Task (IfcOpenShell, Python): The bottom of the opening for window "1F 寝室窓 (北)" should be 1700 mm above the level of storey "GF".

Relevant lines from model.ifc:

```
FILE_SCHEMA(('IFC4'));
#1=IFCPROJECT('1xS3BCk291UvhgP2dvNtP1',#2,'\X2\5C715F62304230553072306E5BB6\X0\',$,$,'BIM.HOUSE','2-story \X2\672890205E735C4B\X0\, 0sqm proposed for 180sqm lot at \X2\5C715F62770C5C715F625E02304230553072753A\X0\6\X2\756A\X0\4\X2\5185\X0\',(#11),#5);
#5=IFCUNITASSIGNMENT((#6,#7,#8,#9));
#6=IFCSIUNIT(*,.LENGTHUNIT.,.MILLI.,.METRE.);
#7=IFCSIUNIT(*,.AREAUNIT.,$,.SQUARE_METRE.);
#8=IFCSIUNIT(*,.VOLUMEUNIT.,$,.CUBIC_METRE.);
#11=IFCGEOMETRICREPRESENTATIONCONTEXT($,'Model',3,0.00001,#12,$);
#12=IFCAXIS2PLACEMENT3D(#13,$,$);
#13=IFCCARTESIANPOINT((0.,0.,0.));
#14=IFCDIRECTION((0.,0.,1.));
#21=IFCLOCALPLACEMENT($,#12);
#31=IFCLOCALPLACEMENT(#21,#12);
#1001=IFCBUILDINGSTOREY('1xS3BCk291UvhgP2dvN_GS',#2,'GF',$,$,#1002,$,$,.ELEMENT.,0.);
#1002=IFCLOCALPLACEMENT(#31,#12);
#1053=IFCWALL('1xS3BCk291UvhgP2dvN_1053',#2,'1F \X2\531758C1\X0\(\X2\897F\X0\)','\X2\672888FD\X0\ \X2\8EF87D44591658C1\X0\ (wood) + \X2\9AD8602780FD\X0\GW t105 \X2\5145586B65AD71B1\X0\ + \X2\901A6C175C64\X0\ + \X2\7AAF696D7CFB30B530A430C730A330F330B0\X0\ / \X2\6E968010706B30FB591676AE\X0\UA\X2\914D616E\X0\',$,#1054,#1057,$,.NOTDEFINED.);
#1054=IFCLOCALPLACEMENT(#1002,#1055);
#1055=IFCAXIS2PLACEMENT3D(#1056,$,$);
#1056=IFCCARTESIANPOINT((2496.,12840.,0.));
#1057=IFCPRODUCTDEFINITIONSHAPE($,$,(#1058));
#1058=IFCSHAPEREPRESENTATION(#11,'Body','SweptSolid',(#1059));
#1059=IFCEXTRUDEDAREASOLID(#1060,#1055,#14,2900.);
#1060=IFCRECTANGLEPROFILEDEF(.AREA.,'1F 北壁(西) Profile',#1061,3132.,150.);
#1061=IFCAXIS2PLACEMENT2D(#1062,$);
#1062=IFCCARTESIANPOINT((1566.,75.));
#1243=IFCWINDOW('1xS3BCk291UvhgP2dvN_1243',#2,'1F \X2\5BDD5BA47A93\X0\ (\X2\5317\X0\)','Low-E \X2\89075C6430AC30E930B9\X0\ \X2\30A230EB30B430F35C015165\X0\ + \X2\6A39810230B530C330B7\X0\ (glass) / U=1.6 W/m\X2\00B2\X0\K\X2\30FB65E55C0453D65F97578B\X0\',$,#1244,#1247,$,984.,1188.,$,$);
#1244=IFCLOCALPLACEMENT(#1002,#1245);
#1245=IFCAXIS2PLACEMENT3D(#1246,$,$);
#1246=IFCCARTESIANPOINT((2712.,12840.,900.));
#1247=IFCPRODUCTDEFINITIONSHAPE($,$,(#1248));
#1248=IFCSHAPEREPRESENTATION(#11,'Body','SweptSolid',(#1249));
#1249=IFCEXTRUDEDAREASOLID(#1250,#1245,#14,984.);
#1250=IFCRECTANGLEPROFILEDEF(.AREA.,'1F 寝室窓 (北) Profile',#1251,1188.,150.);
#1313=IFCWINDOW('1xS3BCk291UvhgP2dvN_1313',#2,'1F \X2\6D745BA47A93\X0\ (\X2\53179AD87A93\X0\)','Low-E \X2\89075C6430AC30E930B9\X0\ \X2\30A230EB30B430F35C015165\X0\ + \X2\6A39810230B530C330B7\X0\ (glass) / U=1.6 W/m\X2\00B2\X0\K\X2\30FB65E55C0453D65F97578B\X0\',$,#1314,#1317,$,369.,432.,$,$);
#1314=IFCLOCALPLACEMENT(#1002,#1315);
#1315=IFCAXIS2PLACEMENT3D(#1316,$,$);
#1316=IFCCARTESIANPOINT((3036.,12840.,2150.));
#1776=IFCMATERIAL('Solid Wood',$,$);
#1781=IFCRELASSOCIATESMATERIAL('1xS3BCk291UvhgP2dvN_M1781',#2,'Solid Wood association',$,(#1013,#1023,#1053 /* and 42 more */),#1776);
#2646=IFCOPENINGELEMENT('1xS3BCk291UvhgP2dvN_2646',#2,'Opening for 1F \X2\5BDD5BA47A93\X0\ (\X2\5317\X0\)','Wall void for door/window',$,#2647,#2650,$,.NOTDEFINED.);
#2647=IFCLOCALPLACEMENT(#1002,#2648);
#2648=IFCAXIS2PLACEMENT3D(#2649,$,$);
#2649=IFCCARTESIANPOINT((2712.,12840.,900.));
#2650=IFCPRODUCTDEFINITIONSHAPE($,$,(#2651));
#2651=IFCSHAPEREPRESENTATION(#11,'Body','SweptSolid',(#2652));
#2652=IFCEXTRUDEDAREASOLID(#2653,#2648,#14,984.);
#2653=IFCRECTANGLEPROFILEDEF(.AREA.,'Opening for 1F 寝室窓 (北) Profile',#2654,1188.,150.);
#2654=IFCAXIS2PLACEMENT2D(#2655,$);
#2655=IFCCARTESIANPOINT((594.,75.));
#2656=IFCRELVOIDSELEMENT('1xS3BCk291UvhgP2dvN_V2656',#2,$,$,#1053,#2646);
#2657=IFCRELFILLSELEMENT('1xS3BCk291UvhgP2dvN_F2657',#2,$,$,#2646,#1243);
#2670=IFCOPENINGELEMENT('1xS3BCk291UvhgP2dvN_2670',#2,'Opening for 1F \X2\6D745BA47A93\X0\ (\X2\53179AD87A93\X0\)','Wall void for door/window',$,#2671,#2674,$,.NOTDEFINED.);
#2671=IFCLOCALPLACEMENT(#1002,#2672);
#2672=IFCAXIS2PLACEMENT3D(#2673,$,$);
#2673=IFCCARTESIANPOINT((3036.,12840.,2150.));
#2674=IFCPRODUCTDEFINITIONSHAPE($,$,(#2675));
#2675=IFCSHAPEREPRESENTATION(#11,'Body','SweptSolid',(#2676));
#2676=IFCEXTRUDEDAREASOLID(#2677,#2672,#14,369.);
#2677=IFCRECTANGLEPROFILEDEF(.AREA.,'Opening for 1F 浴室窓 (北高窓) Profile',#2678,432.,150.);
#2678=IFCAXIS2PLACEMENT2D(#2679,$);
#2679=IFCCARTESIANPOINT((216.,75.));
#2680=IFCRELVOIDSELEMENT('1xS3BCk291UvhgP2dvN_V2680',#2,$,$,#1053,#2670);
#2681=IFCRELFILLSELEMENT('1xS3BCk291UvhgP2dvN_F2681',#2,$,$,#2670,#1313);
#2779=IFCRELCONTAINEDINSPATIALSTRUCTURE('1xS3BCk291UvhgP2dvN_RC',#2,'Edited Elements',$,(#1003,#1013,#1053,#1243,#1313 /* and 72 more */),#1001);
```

```python
import numpy as np
import ifcopenshell
import ifcopenshell.api.geometry
import ifcopenshell.geom
import ifcopenshell.util.element
import ifcopenshell.util.placement
import ifcopenshell.util.shape
import ifcopenshell.util.unit

model = ifcopenshell.open("model.ifc")
unit_scale = ifcopenshell.util.unit.calculate_unit_scale(model)

window = model.by_id(1243)
opening = window.FillsVoids[0].RelatingOpeningElement
storey = ifcopenshell.util.element.get_container(window, ifc_class="IfcBuildingStorey")
level = ifcopenshell.util.placement.get_local_placement(storey.ObjectPlacement)[2, 3]

# The opening's origin need not be at the sill, so measure its lowest point.
shape = ifcopenshell.geom.create_shape(ifcopenshell.geom.settings(), opening)
bottom = ifcopenshell.util.shape.get_shape_bottom_elevation(shape, shape.geometry) / unit_scale
dz = level + 1.7 / unit_scale - bottom

shift = np.array([0.0, 0.0, dz])
# The window is not placed relative to its opening, so move both.
for product in (opening, window):
    matrix = ifcopenshell.util.placement.get_local_placement(product.ObjectPlacement)
    matrix[:3, 3] += shift
    ifcopenshell.api.geometry.edit_object_placement(model, product=product, matrix=matrix, is_si=False)

print(f"moved by {dz * unit_scale:+.3f} m")

model.write("model_edited.ifc")
```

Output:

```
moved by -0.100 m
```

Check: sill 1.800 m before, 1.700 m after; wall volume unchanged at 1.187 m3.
